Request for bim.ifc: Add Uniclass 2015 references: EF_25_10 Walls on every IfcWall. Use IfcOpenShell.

First a look at what the model holds.

```python
import ifcopenshell

model = ifcopenshell.open("bim.ifc")
print(model.schema)
print("classifications:", [c.Name for c in model.by_type("IfcClassification")])
for ifc_class in ("IfcDoor", "IfcRoof", "IfcStair", "IfcWall", "IfcWindow"):
    print(ifc_class, len(model.by_type(ifc_class)))
```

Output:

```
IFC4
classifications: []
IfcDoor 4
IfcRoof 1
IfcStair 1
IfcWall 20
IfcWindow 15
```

```python
import ifcopenshell
import ifcopenshell.api.classification

model = ifcopenshell.open("bim.ifc")

system = ifcopenshell.api.classification.add_classification(model, classification="Uniclass 2015")

codes = {
    "IfcWall": ("EF_25_10", "Walls"),
}
for ifc_class, (code, name) in codes.items():
    products = model.by_type(ifc_class)
    ifcopenshell.api.classification.add_reference(
        model, products=products, classification=system, identification=code, name=name
    )
    print(code, len(products))

model.write("bim-out.ifc")
```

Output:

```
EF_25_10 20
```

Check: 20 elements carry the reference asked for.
